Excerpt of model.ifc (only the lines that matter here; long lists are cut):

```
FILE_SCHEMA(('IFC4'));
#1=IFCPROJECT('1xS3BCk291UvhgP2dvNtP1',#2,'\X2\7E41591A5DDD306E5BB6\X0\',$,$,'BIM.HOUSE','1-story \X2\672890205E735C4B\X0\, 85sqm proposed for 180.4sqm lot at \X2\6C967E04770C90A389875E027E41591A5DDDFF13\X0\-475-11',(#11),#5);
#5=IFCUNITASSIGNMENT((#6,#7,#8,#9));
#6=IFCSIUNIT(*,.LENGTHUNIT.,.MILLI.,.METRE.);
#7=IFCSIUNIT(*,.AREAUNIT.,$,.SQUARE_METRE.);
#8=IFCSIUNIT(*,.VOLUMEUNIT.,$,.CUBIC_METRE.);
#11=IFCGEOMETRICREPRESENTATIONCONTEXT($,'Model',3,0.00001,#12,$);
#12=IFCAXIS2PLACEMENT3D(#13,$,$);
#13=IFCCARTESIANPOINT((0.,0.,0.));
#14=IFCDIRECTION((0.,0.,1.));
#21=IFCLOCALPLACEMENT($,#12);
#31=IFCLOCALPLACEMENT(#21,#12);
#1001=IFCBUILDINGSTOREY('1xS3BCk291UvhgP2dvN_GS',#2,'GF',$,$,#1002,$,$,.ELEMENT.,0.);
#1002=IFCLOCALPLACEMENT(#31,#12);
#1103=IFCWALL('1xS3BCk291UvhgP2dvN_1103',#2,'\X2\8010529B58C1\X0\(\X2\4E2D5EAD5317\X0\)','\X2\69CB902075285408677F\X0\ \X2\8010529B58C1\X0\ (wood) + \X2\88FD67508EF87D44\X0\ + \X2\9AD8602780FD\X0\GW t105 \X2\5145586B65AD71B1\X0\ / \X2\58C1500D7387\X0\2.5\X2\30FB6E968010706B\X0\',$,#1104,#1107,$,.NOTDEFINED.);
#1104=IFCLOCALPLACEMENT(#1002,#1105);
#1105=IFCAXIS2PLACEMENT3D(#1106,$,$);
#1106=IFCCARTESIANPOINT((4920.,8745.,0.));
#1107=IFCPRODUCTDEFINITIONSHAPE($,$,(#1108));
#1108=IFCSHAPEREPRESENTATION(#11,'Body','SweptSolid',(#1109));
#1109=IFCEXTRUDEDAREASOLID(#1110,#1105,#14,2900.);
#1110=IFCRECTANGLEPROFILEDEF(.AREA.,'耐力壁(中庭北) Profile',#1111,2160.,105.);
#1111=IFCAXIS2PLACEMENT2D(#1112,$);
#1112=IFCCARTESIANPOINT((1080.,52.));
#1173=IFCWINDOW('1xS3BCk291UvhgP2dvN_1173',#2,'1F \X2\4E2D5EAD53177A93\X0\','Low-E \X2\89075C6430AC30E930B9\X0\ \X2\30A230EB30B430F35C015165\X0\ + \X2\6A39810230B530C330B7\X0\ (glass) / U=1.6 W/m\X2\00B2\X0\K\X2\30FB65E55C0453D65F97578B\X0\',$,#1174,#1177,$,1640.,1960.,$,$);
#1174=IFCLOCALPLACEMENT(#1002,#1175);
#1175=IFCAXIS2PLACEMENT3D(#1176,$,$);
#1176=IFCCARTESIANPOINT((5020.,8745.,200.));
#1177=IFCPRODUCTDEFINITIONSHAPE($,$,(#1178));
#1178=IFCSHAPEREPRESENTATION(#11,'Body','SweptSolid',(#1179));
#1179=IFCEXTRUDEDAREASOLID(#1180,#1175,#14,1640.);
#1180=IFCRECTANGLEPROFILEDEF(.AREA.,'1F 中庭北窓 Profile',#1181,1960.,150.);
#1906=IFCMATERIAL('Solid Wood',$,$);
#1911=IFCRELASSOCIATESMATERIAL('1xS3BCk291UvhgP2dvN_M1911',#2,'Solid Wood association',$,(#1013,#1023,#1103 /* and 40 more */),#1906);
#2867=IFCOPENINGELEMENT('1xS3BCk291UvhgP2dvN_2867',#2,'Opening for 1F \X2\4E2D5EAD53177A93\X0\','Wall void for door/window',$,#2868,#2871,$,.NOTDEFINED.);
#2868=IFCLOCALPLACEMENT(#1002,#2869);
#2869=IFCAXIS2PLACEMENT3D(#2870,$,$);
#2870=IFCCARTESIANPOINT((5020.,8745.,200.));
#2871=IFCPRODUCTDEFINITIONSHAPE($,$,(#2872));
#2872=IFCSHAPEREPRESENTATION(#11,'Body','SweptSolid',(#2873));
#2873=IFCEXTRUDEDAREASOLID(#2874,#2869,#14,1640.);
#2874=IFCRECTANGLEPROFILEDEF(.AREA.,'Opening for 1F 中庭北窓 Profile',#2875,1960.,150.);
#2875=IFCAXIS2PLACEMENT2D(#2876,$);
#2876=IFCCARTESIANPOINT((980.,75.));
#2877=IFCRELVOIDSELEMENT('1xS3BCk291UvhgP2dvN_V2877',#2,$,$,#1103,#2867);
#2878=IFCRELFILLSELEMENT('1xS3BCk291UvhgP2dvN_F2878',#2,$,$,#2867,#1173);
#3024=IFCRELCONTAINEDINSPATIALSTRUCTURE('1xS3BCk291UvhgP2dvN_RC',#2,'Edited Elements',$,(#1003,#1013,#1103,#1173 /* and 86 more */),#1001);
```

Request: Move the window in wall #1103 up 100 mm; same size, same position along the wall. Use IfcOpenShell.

```python
import numpy as np
import ifcopenshell
import ifcopenshell.api.geometry
import ifcopenshell.util.placement
import ifcopenshell.util.unit

model = ifcopenshell.open("model.ifc")
unit_scale = ifcopenshell.util.unit.calculate_unit_scale(model)

window = model.by_guid("1xS3BCk291UvhgP2dvN_1173")
opening = window.FillsVoids[0].RelatingOpeningElement
dz = 0.1 / unit_scale

shift = np.array([0.0, 0.0, dz])
# The window is not placed relative to its opening, so move both.
for product in (opening, window):
    matrix = ifcopenshell.util.placement.get_local_placement(product.ObjectPlacement)
    matrix[:3, 3] += shift
    ifcopenshell.api.geometry.edit_object_placement(model, product=product, matrix=matrix, is_si=False)

print(f"moved by {dz * unit_scale:+.3f} m")

model.write("model_rev.ifc")
```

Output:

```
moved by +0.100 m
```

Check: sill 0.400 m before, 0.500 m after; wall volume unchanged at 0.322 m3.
